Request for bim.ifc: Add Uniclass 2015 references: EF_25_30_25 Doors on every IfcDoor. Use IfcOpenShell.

First a look at what the model holds.

```python
import ifcopenshell

model = ifcopenshell.open("bim.ifc")
print(model.schema)
print("classifications:", [c.Name for c in model.by_type("IfcClassification")])
for ifc_class in ("IfcDoor", "IfcRoof", "IfcStair", "IfcWall", "IfcWindow"):
    print(ifc_class, len(model.by_type(ifc_class)))
```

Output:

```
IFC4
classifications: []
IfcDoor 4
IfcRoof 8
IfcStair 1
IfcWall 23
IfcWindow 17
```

```python
import ifcopenshell
import ifcopenshell.api.classification

model = ifcopenshell.open("bim.ifc")

system = ifcopenshell.api.classification.add_classification(model, classification="Uniclass 2015")

codes = {
    "IfcDoor": ("EF_25_30_25", "Doors"),
}
for ifc_class, (code, name) in codes.items():
    products = model.by_type(ifc_class)
    ifcopenshell.api.classification.add_reference(
        model, products=products, classification=system, identification=code, name=name
    )
    print(code, len(products))

model.write("bim_rev.ifc")
```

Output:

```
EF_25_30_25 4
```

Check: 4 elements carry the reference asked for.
